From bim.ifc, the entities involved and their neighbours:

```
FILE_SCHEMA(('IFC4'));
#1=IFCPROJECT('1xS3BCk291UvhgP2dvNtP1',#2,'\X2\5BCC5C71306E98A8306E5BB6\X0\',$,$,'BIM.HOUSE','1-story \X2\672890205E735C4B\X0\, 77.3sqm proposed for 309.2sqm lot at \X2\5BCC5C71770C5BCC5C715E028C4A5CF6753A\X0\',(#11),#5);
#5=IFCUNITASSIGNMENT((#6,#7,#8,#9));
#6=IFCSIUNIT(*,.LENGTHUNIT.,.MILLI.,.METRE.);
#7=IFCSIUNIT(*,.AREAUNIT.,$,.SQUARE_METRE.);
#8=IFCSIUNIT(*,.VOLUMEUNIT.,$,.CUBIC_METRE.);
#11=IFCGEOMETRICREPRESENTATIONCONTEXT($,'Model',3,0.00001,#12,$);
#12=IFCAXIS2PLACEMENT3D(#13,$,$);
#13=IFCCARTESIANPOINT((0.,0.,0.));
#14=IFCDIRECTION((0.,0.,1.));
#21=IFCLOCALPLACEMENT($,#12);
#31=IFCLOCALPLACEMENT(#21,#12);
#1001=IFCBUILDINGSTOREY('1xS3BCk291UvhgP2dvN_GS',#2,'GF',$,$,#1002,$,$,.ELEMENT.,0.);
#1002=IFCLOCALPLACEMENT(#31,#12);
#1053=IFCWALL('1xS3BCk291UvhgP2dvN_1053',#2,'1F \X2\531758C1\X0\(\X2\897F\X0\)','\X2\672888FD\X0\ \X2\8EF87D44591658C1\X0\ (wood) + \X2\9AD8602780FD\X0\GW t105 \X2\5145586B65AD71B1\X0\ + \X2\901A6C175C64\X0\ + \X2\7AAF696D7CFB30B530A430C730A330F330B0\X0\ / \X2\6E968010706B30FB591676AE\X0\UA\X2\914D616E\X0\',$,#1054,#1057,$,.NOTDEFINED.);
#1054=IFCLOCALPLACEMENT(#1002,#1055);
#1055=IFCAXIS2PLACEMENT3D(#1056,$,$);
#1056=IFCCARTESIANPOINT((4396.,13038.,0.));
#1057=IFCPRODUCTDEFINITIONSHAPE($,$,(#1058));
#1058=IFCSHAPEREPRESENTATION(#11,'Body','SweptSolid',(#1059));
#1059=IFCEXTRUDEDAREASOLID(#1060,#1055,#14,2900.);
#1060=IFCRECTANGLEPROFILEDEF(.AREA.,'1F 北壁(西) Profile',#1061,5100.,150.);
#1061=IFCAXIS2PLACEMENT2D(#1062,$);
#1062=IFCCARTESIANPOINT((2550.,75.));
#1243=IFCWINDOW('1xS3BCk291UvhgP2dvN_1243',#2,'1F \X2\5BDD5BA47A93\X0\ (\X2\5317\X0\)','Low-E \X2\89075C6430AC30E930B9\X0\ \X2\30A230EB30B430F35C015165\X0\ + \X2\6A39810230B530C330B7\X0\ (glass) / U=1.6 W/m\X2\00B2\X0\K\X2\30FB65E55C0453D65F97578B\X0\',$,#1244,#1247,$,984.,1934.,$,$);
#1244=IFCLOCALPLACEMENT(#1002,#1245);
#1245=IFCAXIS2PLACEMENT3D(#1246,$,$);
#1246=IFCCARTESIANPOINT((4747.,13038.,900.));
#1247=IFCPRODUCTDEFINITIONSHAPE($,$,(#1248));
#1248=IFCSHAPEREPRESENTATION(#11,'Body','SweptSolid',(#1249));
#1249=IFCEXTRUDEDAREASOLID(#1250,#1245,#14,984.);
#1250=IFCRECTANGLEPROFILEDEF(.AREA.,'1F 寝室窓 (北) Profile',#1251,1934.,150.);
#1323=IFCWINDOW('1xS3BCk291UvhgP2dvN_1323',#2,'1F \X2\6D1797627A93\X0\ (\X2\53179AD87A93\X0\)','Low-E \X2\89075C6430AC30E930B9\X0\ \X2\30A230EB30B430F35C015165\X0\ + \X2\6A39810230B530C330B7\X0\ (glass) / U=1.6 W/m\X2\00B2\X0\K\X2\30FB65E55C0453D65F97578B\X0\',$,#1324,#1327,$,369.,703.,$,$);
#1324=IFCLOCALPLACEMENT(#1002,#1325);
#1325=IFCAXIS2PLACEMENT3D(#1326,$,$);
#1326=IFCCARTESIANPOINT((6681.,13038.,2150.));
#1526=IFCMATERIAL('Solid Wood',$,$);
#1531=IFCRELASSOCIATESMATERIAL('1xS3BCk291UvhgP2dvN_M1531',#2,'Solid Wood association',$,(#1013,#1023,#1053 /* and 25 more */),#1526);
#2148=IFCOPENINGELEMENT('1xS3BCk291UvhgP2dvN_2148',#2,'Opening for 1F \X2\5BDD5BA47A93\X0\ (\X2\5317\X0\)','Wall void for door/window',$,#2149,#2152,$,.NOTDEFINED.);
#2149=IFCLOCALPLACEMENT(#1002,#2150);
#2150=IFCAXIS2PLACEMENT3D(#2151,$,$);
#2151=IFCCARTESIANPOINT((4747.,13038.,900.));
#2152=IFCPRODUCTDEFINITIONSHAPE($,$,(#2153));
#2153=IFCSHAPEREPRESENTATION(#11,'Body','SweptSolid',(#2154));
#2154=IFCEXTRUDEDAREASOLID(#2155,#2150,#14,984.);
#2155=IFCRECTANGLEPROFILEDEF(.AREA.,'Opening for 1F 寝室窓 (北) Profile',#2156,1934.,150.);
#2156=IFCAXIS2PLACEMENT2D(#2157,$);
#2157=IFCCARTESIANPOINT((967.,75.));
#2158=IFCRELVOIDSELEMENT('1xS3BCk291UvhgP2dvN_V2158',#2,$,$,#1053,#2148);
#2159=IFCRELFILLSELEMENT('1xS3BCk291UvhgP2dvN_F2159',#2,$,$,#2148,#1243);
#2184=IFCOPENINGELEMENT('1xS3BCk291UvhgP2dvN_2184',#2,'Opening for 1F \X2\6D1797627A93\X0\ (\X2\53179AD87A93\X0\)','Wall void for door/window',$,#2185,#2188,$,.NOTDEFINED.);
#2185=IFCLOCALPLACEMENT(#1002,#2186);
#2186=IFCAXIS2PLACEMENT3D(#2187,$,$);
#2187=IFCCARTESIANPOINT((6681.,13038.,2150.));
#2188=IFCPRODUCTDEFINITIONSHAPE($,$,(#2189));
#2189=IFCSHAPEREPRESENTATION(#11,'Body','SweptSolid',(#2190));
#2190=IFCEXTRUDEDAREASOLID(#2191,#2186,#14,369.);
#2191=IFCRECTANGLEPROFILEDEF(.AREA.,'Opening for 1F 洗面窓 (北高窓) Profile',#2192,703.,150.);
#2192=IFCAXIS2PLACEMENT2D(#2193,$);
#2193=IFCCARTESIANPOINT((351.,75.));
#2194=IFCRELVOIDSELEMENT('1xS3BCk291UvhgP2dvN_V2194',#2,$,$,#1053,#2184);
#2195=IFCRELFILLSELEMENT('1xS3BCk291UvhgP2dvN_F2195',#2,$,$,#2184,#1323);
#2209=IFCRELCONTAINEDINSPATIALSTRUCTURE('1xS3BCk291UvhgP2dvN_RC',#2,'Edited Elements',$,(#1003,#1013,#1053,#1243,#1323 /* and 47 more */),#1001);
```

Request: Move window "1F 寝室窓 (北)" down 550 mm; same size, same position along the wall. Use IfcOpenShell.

```python
import numpy as np
import ifcopenshell
import ifcopenshell.api.geometry
import ifcopenshell.util.placement
import ifcopenshell.util.unit

model = ifcopenshell.open("bim.ifc")
unit_scale = ifcopenshell.util.unit.calculate_unit_scale(model)

window = model.by_guid("1xS3BCk291UvhgP2dvN_1243")
opening = window.FillsVoids[0].RelatingOpeningElement
dz = -0.55 / unit_scale

shift = np.array([0.0, 0.0, dz])
# The window is not placed relative to its opening, so move both.
for product in (opening, window):
    matrix = ifcopenshell.util.placement.get_local_placement(product.ObjectPlacement)
    matrix[:3, 3] += shift
    ifcopenshell.api.geometry.edit_object_placement(model, product=product, matrix=matrix, is_si=False)

print(f"moved by {dz * unit_scale:+.3f} m")

model.write("bim_edited.ifc")
```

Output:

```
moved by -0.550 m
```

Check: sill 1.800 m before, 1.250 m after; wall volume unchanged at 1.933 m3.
